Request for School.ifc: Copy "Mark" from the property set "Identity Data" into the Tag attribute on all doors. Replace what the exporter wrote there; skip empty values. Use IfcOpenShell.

First a look at what the model holds.

```python
import ifcopenshell
import ifcopenshell.util.element

model = ifcopenshell.open("School.ifc")
print(model.schema)
doors = model.by_type("IfcDoor")
print(len(doors), "doors")
for e in doors[:8]:
    source = ifcopenshell.util.element.get_pset(e, "Identity Data", "Mark")
    target = e.Tag
    print(e.id(), repr(source), repr(target), sep=" | ")
```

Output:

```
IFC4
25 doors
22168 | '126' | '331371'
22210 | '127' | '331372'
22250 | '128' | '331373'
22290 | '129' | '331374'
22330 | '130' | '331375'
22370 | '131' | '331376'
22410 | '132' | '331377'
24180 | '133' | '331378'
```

```python
import ifcopenshell
import ifcopenshell.util.element

model = ifcopenshell.open("School.ifc")

count = 0
for e in model.by_type("IfcDoor"):
    value = ifcopenshell.util.element.get_pset(e, "Identity Data", "Mark")
    current = e.Tag
    if not value or not value.strip() or current == value:
        continue
    e.Tag = value
    count += 1

print(count, "doors updated")

model.write("School_updated.ifc")
```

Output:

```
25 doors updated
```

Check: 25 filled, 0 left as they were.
